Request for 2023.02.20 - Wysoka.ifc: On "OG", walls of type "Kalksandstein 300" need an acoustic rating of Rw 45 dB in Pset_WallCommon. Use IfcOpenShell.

First a look at what the model holds.

```python
import ifcopenshell
import ifcopenshell.util.element

model = ifcopenshell.open("2023.02.20 - Wysoka.ifc")
print(model.schema)
storey = next(s for s in model.by_type("IfcBuildingStorey") if s.Name == "OG")
walls = [e for e in ifcopenshell.util.element.get_decomposition(storey) if e.is_a("IfcWall")]
seen = {}
for e in walls:
    element_type = ifcopenshell.util.element.get_type(e)
    key = (element_type.Name if element_type != e and element_type else None, ifcopenshell.util.element.get_pset(e, "Pset_WallCommon", "AcousticRating"))
    seen[key] = seen.get(key, 0) + 1
for (name, value), count in sorted(seen.items(), key=str):
    print(count, "x", name, "|", value)
```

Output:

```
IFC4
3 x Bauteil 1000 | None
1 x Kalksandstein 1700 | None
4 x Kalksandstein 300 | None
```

```python
import ifcopenshell
import ifcopenshell.api.pset
import ifcopenshell.util.element

model = ifcopenshell.open("2023.02.20 - Wysoka.ifc")

storey = next(s for s in model.by_type("IfcBuildingStorey") if s.Name == "OG")
walls = [e for e in ifcopenshell.util.element.get_decomposition(storey) if e.is_a("IfcWall")]

count = 0
for e in walls:
    element_type = ifcopenshell.util.element.get_type(e)
    if element_type in (None, e) or element_type.Name != "Kalksandstein 300":
        continue
    # add_pset returns the element's existing set when there is one.
    pset = ifcopenshell.api.pset.add_pset(model, product=e, name="Pset_WallCommon")
    ifcopenshell.api.pset.edit_pset(model, pset=pset, properties={"AcousticRating": "Rw 45 dB"})
    count += 1

print(count, "walls updated")

model.write("2023.02.20 - Wysoka_updated.ifc")
```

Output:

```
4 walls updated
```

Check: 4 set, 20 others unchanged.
